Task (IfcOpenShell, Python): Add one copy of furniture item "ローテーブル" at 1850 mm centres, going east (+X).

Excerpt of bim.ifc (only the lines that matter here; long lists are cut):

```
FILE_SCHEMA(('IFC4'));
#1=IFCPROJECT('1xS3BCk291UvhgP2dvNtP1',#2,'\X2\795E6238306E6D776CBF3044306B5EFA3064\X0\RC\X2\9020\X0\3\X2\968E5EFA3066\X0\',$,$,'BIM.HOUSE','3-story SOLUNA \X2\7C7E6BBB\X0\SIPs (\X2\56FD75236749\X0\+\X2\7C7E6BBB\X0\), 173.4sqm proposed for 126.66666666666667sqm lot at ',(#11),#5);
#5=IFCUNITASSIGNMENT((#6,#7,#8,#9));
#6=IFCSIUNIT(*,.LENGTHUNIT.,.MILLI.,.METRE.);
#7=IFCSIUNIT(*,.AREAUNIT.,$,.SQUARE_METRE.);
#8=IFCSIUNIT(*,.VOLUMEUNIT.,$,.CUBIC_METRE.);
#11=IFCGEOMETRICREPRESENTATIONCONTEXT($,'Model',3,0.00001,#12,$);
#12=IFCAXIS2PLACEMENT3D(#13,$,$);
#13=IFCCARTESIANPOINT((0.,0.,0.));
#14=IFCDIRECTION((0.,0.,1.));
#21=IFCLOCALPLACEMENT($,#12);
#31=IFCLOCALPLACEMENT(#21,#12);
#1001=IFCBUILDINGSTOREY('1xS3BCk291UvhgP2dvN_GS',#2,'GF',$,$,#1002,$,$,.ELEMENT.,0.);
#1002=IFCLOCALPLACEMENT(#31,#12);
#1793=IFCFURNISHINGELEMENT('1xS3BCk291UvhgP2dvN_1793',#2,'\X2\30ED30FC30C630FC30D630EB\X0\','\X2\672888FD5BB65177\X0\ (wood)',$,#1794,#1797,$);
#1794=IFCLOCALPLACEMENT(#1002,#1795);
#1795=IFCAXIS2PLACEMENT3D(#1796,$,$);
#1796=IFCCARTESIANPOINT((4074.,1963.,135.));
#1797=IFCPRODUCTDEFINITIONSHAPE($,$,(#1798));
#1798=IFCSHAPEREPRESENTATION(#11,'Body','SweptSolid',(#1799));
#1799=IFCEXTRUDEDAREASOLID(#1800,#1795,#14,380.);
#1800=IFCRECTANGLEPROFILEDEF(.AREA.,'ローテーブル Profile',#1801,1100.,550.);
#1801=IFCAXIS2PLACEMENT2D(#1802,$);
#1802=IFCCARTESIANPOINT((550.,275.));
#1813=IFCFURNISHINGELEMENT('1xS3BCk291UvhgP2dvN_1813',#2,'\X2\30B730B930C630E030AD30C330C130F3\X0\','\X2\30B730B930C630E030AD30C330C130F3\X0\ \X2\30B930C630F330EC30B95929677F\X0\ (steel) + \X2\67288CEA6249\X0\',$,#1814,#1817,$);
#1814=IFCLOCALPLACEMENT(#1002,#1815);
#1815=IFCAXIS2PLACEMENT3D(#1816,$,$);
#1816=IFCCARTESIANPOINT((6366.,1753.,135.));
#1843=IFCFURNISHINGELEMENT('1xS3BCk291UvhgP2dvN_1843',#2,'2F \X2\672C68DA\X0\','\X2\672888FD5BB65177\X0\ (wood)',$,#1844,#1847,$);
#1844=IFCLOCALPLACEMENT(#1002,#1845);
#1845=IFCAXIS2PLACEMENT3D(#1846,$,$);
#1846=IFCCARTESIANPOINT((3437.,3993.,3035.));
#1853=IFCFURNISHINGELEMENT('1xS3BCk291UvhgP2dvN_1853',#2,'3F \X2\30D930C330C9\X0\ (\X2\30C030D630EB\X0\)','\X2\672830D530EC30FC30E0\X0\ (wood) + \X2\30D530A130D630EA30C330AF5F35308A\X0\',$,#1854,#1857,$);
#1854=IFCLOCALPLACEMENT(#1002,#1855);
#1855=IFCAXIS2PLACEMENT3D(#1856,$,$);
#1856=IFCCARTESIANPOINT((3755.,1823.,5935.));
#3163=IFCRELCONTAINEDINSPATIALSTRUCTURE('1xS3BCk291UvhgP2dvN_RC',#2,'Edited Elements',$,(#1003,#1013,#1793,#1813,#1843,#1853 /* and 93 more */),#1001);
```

```python
import numpy as np
import ifcopenshell
import ifcopenshell.api.geometry
import ifcopenshell.api.root
import ifcopenshell.util.element
import ifcopenshell.util.placement
import ifcopenshell.util.unit

model = ifcopenshell.open("bim.ifc")
unit_scale = ifcopenshell.util.unit.calculate_unit_scale(model)


def reuse_history(source, copy):
    """copy_class also copies each property set's owner history, people and application; keep the originals."""
    for rel in copy.IsDefinedBy:
        if rel.is_a("IfcRelDefinesByProperties") and (history := rel.RelatingPropertyDefinition.OwnerHistory):
            rel.RelatingPropertyDefinition.OwnerHistory = source.OwnerHistory
            ifcopenshell.util.element.remove_deep2(model, history)


source = model.by_guid("1xS3BCk291UvhgP2dvN_1793")
base = ifcopenshell.util.placement.get_local_placement(source.ObjectPlacement)
step = np.array([1.0, 0.0, 0.0]) * 1.85 / unit_scale

for i in range(1, 2):
    copy = ifcopenshell.api.root.copy_class(model, product=source)
    copy.Representation = ifcopenshell.util.element.copy_deep(
        model, source.Representation, exclude=["IfcGeometricRepresentationContext", "IfcRepresentationMap"]
    )
    reuse_history(source, copy)
    matrix = base.copy()
    matrix[:3, 3] += i * step
    print("added at", matrix[:3, 3].round(3) + 0.0)
    ifcopenshell.api.geometry.edit_object_placement(model, product=copy, matrix=matrix, is_si=False)

model.write("bim_rev.ifc")
```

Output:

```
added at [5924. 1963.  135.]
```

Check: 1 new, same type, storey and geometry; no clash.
